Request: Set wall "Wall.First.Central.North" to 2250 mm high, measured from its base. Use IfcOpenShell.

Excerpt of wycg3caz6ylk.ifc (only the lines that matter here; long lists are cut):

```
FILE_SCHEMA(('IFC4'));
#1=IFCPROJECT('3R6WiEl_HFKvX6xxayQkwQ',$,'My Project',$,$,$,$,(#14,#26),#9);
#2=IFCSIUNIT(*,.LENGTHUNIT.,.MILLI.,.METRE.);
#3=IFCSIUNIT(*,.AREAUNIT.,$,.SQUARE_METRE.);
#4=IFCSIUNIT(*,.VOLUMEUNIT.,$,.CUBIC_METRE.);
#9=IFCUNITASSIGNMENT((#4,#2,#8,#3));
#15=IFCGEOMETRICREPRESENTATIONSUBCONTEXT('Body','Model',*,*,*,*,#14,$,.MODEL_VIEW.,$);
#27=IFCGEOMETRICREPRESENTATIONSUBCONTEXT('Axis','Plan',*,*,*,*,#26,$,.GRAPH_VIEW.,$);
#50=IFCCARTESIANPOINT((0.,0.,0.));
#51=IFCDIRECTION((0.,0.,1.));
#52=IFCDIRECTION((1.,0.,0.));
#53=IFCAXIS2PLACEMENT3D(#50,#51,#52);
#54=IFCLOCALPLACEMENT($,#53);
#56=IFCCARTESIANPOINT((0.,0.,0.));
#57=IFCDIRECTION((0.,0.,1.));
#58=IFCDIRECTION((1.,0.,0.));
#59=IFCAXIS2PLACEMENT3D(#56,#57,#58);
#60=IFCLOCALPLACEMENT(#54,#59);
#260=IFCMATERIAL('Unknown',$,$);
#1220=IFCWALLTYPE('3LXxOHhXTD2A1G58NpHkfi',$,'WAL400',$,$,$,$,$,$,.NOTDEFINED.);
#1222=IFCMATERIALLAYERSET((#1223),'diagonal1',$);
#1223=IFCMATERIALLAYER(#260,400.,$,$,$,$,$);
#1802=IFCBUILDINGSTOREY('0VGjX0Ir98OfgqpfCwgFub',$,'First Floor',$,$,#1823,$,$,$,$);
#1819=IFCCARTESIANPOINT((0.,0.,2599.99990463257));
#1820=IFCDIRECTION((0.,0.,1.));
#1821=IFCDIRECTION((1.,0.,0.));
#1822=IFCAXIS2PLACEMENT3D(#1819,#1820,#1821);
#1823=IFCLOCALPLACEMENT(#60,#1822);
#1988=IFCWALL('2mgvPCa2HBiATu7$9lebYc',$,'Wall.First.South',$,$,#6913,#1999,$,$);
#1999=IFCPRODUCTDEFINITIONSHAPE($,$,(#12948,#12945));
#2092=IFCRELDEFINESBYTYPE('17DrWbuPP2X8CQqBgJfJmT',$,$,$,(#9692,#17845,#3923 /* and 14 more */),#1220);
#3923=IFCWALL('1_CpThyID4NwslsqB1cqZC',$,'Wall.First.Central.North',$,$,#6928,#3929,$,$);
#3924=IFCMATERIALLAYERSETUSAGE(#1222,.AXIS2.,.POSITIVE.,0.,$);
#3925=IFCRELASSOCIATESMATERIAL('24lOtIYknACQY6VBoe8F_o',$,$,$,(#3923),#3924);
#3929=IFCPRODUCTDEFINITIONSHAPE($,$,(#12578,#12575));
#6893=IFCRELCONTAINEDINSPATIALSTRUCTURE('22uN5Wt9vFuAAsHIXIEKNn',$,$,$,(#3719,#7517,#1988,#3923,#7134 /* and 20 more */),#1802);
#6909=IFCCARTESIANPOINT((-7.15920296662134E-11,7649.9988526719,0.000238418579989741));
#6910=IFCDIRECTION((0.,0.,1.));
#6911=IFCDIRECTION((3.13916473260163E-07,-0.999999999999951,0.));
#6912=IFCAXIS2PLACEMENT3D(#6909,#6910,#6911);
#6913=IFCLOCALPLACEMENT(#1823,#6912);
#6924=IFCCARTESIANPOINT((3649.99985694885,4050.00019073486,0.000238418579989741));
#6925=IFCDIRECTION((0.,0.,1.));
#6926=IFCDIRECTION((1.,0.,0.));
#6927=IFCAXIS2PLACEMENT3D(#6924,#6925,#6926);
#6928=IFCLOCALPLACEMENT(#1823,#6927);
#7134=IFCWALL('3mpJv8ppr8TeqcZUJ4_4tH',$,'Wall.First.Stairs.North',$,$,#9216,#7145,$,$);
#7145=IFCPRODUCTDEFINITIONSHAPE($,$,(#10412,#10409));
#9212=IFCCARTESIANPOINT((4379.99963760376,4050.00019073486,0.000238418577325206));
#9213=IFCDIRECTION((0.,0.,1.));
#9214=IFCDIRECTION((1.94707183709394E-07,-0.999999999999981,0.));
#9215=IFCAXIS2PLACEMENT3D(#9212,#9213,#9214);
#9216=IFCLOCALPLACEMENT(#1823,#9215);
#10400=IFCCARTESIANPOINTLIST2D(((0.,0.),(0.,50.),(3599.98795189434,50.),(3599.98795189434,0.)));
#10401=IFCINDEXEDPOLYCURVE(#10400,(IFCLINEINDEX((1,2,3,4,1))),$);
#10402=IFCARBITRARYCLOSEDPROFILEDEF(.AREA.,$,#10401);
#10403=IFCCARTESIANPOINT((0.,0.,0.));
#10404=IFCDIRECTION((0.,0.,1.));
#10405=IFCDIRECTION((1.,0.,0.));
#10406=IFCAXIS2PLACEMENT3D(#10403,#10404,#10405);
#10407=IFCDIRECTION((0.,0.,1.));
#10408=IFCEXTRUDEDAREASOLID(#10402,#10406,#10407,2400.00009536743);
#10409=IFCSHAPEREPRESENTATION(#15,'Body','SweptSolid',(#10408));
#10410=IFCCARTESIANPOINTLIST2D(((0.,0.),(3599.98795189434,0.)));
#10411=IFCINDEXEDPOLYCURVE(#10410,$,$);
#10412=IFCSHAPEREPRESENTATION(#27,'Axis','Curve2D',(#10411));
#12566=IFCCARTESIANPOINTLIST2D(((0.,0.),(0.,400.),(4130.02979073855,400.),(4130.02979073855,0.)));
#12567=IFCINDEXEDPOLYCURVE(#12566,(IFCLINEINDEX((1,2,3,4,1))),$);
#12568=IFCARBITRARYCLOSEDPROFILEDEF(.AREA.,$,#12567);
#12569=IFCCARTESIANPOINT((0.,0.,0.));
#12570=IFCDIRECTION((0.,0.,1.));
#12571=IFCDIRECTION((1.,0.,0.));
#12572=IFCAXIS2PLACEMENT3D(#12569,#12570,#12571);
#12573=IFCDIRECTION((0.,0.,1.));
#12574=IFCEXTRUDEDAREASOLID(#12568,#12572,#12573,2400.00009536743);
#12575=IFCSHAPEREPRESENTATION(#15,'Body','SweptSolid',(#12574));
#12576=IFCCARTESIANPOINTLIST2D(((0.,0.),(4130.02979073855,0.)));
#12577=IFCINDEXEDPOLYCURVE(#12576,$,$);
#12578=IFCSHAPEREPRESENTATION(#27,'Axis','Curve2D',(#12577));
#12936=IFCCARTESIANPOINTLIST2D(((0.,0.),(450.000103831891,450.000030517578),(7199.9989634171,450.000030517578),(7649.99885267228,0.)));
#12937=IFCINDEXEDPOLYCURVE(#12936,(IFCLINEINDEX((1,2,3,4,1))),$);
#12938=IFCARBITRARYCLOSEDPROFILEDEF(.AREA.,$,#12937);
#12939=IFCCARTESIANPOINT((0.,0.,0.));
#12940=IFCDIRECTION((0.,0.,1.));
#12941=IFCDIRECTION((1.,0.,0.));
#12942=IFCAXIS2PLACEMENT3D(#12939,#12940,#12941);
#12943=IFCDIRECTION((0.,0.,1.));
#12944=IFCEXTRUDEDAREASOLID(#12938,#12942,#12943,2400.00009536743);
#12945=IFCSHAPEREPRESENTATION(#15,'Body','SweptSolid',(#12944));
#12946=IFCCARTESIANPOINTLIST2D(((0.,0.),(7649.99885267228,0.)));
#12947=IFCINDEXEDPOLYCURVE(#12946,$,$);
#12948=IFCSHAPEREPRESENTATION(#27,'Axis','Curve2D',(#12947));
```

```python
import ifcopenshell
import ifcopenshell.geom
import ifcopenshell.util.representation
import ifcopenshell.util.shape

model = ifcopenshell.open("wycg3caz6ylk.ifc")
settings = ifcopenshell.geom.settings()


def volume(element):
    """Net volume in cubic metres, openings subtracted."""
    shape = ifcopenshell.geom.create_shape(settings, element)
    return ifcopenshell.util.shape.get_volume(shape.geometry)


wall = model.by_id(3923)
before = volume(wall)

body = ifcopenshell.util.representation.get_representation(wall, "Model", "Body")
solid = body.Items[0]
old_height = solid.Depth
solid.Depth = 2250.0
after = volume(wall)

print(f"height {old_height:g} -> {solid.Depth:g}, volume {before:.3f} -> {after:.3f} m3")

model.write("wycg3caz6ylk_v2.ifc")
```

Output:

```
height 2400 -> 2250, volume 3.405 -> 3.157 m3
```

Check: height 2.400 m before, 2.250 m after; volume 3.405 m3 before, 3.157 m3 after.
